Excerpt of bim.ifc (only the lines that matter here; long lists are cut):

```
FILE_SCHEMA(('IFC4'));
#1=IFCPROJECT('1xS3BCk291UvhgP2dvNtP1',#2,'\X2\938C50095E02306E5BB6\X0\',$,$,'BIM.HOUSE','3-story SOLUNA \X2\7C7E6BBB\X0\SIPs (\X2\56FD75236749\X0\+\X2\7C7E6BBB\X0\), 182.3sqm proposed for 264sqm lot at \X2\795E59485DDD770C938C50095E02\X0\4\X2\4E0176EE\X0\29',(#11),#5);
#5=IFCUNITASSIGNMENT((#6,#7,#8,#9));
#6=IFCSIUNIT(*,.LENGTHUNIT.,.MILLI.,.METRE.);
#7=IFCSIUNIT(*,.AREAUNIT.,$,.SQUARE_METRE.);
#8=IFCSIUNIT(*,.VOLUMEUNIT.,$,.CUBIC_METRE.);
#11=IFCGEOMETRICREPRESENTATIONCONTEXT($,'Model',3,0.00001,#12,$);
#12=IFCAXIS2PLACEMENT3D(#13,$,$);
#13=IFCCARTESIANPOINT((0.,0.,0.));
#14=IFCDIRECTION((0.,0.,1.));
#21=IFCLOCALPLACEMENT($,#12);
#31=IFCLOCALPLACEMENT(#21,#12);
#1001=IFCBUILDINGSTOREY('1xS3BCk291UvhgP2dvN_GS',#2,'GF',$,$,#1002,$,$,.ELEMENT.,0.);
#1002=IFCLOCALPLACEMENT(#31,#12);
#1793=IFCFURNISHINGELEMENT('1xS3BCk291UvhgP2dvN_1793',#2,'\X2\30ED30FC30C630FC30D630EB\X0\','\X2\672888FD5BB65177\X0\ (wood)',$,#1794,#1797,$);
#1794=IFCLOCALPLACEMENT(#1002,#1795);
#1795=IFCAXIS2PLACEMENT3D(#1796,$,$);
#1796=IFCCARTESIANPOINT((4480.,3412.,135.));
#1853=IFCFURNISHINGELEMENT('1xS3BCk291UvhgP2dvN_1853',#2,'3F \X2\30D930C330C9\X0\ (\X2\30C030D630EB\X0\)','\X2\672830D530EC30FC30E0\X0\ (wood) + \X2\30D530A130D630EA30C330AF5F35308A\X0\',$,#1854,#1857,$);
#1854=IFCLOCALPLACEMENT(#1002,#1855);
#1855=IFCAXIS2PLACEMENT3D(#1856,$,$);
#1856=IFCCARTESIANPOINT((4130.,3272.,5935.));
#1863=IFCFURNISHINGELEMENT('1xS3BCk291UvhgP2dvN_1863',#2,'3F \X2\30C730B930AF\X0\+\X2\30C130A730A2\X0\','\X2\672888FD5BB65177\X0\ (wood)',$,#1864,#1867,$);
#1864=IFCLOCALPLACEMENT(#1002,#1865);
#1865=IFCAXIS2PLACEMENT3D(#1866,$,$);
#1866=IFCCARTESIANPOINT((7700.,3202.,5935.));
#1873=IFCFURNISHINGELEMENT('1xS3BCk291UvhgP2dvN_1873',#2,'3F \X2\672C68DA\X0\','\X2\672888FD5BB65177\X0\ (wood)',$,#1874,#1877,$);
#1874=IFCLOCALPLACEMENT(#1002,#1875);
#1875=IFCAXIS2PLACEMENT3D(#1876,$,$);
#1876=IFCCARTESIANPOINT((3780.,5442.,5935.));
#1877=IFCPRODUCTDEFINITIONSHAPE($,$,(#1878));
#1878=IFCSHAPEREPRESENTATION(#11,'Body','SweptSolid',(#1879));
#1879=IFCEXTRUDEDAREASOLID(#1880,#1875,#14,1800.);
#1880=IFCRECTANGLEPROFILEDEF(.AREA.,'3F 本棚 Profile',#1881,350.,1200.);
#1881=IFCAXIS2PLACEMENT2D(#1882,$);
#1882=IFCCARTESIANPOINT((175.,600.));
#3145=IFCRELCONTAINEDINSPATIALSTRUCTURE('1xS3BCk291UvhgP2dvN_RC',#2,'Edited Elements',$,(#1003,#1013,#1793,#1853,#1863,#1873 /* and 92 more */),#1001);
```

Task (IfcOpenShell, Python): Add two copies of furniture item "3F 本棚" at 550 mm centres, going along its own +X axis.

```python
import ifcopenshell
import ifcopenshell.api.geometry
import ifcopenshell.api.root
import ifcopenshell.util.element
import ifcopenshell.util.placement

model = ifcopenshell.open("bim.ifc")


def reuse_history(source, copy):
    """copy_class also copies each property set's owner history, people and application; keep the originals."""
    for rel in copy.IsDefinedBy:
        if rel.is_a("IfcRelDefinesByProperties") and (history := rel.RelatingPropertyDefinition.OwnerHistory):
            rel.RelatingPropertyDefinition.OwnerHistory = source.OwnerHistory
            ifcopenshell.util.element.remove_deep2(model, history)


source = model.by_id(1873)
base = ifcopenshell.util.placement.get_local_placement(source.ObjectPlacement)
step = base[:3, 0] * 550.0

for i in range(1, 3):
    copy = ifcopenshell.api.root.copy_class(model, product=source)
    copy.Representation = ifcopenshell.util.element.copy_deep(
        model, source.Representation, exclude=["IfcGeometricRepresentationContext", "IfcRepresentationMap"]
    )
    reuse_history(source, copy)
    matrix = base.copy()
    matrix[:3, 3] += i * step
    print("added at", matrix[:3, 3].round(3) + 0.0)
    ifcopenshell.api.geometry.edit_object_placement(model, product=copy, matrix=matrix, is_si=False)

model.write("bim_v2.ifc")
```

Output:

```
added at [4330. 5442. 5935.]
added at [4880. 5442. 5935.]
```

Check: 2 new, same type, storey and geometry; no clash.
